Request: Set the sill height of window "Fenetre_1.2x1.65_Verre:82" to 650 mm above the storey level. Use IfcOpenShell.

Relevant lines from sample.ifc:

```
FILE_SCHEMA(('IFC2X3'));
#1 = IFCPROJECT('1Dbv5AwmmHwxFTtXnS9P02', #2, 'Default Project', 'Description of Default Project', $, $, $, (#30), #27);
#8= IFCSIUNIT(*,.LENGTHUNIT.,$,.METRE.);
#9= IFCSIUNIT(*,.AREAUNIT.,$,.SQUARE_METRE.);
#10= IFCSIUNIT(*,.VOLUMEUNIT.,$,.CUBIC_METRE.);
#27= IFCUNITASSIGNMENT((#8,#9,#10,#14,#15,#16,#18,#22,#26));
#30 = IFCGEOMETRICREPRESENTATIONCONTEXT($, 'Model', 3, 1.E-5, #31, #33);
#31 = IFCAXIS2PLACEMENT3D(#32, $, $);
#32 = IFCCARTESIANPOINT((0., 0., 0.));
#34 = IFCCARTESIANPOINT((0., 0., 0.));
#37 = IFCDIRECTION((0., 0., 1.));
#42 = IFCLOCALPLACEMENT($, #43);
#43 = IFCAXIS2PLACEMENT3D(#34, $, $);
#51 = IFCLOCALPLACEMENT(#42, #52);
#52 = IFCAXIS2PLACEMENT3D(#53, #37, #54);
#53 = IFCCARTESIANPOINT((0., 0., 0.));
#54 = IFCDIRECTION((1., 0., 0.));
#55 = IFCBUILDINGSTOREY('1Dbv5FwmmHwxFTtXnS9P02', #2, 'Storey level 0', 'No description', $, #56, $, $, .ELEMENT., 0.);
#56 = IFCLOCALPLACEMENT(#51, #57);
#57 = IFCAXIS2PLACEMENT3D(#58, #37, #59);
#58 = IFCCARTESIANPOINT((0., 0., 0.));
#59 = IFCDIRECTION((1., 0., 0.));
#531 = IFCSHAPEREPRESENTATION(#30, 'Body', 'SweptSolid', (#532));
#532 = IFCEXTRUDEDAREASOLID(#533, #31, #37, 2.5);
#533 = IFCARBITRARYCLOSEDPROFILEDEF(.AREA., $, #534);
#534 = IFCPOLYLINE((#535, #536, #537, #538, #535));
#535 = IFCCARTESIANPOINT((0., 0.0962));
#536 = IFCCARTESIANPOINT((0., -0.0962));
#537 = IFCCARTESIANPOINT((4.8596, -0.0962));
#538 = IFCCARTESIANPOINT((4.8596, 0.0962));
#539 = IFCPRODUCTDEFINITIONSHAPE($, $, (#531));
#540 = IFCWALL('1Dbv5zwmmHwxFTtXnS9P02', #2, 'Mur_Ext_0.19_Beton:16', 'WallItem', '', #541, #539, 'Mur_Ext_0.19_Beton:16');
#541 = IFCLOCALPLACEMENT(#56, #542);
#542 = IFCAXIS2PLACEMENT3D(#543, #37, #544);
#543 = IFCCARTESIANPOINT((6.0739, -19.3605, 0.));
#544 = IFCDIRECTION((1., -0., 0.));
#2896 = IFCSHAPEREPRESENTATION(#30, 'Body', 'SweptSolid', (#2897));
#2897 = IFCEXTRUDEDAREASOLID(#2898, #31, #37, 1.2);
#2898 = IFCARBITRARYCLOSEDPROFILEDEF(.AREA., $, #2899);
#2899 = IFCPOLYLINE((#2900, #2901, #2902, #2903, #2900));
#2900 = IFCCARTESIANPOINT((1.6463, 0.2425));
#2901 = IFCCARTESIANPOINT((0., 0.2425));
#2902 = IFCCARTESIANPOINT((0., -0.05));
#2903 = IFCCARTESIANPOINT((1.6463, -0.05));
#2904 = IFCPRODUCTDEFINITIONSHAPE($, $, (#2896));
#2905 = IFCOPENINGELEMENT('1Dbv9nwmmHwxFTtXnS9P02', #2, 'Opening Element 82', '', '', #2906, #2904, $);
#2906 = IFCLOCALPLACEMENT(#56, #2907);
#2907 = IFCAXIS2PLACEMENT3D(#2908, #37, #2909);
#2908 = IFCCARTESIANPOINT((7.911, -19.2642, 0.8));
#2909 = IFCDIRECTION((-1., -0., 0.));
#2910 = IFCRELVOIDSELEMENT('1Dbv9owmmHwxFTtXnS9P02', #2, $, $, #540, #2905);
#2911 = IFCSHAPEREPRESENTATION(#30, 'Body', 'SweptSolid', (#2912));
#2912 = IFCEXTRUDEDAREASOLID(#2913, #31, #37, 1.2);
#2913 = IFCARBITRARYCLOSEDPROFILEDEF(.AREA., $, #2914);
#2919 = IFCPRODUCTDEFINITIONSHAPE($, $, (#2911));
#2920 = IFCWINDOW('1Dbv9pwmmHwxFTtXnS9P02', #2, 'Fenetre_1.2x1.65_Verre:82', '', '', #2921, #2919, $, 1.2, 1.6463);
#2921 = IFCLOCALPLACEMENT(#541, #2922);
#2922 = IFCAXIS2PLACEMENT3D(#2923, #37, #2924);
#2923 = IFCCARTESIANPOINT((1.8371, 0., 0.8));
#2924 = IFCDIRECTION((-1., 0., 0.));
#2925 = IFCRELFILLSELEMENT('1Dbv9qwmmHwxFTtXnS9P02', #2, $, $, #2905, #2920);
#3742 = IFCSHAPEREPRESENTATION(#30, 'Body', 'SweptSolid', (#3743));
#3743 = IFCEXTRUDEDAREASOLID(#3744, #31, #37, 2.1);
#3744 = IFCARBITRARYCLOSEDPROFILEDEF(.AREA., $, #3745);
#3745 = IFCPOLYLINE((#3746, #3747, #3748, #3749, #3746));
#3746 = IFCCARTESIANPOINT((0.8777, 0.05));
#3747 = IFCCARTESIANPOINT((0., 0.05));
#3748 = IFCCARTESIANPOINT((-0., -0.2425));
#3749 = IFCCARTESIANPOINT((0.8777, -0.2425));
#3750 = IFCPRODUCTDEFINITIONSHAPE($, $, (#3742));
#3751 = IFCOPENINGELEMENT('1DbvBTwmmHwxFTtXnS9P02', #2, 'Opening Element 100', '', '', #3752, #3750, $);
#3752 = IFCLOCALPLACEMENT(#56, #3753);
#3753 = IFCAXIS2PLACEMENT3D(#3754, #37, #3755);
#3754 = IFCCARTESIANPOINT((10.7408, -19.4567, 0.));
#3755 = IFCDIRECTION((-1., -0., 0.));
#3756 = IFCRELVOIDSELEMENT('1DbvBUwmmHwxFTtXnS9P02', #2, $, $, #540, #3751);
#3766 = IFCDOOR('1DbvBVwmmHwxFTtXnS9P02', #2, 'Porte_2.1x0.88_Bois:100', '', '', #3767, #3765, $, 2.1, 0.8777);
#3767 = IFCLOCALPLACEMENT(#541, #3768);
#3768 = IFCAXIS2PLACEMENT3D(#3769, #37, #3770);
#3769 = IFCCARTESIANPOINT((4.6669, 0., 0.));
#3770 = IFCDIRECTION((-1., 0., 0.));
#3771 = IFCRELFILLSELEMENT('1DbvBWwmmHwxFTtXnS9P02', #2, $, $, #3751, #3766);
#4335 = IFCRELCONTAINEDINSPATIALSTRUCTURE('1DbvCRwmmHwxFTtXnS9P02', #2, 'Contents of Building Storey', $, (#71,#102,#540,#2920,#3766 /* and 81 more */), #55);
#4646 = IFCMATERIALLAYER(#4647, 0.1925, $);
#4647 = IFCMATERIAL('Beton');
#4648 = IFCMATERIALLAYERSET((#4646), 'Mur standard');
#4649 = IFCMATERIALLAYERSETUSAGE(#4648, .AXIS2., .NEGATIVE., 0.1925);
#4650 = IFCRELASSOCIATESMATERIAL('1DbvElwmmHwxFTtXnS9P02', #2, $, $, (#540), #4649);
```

```python
import numpy as np
import ifcopenshell
import ifcopenshell.api.geometry
import ifcopenshell.geom
import ifcopenshell.util.element
import ifcopenshell.util.placement
import ifcopenshell.util.shape
import ifcopenshell.util.unit

model = ifcopenshell.open("sample.ifc")
unit_scale = ifcopenshell.util.unit.calculate_unit_scale(model)

window = model.by_guid("1Dbv9pwmmHwxFTtXnS9P02")
opening = window.FillsVoids[0].RelatingOpeningElement
storey = ifcopenshell.util.element.get_container(window, ifc_class="IfcBuildingStorey")
level = ifcopenshell.util.placement.get_local_placement(storey.ObjectPlacement)[2, 3]

# The opening's origin need not be at the sill, so measure its lowest point.
shape = ifcopenshell.geom.create_shape(ifcopenshell.geom.settings(), opening)
bottom = ifcopenshell.util.shape.get_shape_bottom_elevation(shape, shape.geometry) / unit_scale
dz = level + 0.65 / unit_scale - bottom

shift = np.array([0.0, 0.0, dz])
# The window is not placed relative to its opening, so move both.
for product in (opening, window):
    matrix = ifcopenshell.util.placement.get_local_placement(product.ObjectPlacement)
    matrix[:3, 3] += shift
    ifcopenshell.api.geometry.edit_object_placement(model, product=product, matrix=matrix, is_si=False)

print(f"moved by {dz * unit_scale:+.3f} m")

model.write("sample_edited.ifc")
```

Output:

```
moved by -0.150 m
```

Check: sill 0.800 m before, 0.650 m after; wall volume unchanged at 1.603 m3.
